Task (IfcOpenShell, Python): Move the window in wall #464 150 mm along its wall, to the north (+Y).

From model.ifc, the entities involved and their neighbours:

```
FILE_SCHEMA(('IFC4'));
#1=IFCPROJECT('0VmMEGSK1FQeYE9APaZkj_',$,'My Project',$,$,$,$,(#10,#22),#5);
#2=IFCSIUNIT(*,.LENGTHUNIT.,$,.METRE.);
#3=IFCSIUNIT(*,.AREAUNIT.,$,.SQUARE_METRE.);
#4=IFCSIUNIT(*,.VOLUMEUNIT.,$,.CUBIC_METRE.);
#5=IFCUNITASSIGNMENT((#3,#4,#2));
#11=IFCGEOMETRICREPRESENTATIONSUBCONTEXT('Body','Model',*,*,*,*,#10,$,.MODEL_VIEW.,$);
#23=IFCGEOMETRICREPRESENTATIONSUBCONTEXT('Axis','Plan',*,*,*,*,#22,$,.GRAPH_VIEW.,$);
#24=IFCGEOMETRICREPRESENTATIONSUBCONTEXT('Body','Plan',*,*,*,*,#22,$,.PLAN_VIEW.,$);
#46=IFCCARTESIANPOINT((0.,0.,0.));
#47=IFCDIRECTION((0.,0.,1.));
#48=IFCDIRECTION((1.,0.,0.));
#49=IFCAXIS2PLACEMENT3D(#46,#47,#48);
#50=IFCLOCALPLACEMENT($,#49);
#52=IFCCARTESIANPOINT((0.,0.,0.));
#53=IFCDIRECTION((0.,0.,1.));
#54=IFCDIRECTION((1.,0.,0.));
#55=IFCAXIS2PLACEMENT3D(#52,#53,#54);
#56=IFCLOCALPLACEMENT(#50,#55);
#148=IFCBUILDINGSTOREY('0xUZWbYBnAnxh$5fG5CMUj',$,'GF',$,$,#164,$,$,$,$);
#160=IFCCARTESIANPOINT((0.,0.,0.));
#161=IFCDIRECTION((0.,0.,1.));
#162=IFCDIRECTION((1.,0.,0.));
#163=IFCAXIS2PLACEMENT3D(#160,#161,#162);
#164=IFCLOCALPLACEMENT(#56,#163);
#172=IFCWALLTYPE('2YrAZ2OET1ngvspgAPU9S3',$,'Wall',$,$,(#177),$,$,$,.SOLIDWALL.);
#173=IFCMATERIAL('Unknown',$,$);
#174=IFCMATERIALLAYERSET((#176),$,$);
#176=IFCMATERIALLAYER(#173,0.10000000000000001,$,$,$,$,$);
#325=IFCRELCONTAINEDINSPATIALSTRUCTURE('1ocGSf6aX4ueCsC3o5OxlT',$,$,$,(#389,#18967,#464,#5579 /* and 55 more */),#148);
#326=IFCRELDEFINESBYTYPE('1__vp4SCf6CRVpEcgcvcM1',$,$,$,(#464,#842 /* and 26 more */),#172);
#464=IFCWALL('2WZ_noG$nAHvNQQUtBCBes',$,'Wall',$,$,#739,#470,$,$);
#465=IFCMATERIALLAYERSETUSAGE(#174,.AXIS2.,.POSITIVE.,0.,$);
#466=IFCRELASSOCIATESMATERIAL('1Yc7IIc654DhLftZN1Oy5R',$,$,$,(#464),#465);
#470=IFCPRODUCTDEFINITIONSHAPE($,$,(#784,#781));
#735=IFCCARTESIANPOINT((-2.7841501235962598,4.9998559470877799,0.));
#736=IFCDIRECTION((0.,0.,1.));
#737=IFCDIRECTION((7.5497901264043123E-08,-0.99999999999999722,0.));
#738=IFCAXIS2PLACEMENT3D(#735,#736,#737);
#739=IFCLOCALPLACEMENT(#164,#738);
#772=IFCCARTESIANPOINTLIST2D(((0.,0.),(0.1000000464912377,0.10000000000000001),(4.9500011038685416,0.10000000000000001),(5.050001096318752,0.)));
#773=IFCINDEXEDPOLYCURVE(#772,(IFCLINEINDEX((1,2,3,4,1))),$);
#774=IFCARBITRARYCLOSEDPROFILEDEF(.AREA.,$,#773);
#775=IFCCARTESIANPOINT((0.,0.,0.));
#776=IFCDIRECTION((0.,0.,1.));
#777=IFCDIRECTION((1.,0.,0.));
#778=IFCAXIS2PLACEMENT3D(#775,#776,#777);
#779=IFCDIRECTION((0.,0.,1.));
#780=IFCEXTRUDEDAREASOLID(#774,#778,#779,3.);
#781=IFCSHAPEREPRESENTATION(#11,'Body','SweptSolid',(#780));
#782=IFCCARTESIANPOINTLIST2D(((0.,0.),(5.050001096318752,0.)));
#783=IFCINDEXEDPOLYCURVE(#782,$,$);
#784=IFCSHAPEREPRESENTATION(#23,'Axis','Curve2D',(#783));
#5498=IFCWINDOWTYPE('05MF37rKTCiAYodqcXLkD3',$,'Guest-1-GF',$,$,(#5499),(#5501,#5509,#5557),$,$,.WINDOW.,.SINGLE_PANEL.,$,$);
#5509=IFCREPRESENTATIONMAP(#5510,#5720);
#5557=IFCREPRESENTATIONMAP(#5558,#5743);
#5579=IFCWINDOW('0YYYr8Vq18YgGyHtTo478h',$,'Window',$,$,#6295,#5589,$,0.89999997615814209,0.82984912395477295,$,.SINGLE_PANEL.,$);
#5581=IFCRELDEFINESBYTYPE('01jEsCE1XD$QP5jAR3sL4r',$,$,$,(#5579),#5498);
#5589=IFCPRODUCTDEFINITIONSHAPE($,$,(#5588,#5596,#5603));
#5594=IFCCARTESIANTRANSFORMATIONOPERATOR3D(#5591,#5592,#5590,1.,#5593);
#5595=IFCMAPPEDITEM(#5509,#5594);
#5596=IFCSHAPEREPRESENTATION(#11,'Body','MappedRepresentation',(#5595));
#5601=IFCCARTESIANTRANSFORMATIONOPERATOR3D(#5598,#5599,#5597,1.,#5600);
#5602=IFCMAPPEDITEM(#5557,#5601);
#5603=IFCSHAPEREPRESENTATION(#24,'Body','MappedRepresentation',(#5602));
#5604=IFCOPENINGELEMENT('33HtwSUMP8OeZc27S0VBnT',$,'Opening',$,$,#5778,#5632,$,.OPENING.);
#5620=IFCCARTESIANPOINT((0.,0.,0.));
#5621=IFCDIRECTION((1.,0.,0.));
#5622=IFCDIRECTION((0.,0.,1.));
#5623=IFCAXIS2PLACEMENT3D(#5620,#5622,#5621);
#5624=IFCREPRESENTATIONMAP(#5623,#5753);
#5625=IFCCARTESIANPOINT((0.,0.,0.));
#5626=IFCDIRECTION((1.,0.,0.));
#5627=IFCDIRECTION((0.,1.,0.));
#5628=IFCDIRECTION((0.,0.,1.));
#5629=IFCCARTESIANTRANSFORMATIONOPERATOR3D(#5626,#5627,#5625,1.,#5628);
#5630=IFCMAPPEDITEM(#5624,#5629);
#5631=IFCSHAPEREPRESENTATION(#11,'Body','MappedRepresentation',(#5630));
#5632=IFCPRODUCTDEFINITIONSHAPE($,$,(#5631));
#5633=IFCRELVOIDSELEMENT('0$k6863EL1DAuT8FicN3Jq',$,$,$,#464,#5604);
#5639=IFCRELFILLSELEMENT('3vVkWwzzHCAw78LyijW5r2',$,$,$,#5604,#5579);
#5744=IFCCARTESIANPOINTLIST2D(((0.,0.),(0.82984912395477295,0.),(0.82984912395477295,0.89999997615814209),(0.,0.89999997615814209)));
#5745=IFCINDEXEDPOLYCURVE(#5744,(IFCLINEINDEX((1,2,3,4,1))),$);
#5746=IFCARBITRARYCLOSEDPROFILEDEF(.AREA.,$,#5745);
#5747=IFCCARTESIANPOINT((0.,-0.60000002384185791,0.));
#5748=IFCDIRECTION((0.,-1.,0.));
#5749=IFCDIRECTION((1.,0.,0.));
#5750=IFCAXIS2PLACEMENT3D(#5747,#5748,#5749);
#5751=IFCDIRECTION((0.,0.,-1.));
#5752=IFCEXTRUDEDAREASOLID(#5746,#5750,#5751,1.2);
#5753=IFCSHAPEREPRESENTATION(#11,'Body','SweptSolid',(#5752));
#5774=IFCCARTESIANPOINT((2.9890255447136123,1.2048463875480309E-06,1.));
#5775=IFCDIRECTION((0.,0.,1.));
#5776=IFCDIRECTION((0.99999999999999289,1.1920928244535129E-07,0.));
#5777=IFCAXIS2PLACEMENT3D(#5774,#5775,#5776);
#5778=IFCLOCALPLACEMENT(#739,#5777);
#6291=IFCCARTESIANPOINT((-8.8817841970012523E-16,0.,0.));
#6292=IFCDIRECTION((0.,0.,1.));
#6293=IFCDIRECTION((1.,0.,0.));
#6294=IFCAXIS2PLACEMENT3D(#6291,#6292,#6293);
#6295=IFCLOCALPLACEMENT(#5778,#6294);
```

```python
import ifcopenshell
import ifcopenshell.api.geometry
import ifcopenshell.util.placement
import ifcopenshell.util.unit

model = ifcopenshell.open("model.ifc")
unit_scale = ifcopenshell.util.unit.calculate_unit_scale(model)

window = model.by_guid("0YYYr8Vq18YgGyHtTo478h")
opening = window.FillsVoids[0].RelatingOpeningElement
wall = opening.VoidsElements[0].RelatingBuildingElement

wall_matrix = ifcopenshell.util.placement.get_local_placement(wall.ObjectPlacement)
shift = wall_matrix[:3, 0] * -0.15 / unit_scale
before = ifcopenshell.util.placement.get_local_placement(window.ObjectPlacement)[:3, 3].copy()

# The window is placed relative to its opening, so it follows when the opening moves.
matrix = ifcopenshell.util.placement.get_local_placement(opening.ObjectPlacement)
matrix[:3, 3] += shift
ifcopenshell.api.geometry.edit_object_placement(
    model, product=opening, matrix=matrix, is_si=False, should_transform_children=True
)

after = ifcopenshell.util.placement.get_local_placement(window.ObjectPlacement)[:3, 3]
print("window moved by", (after - before).round(3) + 0.0)

model.write("model_updated.ifc")
```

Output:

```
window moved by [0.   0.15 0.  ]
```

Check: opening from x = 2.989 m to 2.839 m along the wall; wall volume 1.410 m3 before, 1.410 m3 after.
